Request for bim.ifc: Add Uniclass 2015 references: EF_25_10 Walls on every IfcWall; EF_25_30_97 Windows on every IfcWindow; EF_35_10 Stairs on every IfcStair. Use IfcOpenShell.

First a look at what the model holds.

```python
import ifcopenshell

model = ifcopenshell.open("bim.ifc")
print(model.schema)
print("classifications:", [c.Name for c in model.by_type("IfcClassification")])
for ifc_class in ("IfcDoor", "IfcRoof", "IfcStair", "IfcWall", "IfcWindow"):
    print(ifc_class, len(model.by_type(ifc_class)))
```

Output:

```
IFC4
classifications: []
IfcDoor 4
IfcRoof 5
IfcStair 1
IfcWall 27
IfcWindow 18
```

```python
import ifcopenshell
import ifcopenshell.api.classification

model = ifcopenshell.open("bim.ifc")

system = ifcopenshell.api.classification.add_classification(model, classification="Uniclass 2015")

codes = {
    "IfcWall": ("EF_25_10", "Walls"),
    "IfcWindow": ("EF_25_30_97", "Windows"),
    "IfcStair": ("EF_35_10", "Stairs"),
}
for ifc_class, (code, name) in codes.items():
    products = model.by_type(ifc_class)
    ifcopenshell.api.classification.add_reference(
        model, products=products, classification=system, identification=code, name=name
    )
    print(code, len(products))

model.write("bim_v2.ifc")
```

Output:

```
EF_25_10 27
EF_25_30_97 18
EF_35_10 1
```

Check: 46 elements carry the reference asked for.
